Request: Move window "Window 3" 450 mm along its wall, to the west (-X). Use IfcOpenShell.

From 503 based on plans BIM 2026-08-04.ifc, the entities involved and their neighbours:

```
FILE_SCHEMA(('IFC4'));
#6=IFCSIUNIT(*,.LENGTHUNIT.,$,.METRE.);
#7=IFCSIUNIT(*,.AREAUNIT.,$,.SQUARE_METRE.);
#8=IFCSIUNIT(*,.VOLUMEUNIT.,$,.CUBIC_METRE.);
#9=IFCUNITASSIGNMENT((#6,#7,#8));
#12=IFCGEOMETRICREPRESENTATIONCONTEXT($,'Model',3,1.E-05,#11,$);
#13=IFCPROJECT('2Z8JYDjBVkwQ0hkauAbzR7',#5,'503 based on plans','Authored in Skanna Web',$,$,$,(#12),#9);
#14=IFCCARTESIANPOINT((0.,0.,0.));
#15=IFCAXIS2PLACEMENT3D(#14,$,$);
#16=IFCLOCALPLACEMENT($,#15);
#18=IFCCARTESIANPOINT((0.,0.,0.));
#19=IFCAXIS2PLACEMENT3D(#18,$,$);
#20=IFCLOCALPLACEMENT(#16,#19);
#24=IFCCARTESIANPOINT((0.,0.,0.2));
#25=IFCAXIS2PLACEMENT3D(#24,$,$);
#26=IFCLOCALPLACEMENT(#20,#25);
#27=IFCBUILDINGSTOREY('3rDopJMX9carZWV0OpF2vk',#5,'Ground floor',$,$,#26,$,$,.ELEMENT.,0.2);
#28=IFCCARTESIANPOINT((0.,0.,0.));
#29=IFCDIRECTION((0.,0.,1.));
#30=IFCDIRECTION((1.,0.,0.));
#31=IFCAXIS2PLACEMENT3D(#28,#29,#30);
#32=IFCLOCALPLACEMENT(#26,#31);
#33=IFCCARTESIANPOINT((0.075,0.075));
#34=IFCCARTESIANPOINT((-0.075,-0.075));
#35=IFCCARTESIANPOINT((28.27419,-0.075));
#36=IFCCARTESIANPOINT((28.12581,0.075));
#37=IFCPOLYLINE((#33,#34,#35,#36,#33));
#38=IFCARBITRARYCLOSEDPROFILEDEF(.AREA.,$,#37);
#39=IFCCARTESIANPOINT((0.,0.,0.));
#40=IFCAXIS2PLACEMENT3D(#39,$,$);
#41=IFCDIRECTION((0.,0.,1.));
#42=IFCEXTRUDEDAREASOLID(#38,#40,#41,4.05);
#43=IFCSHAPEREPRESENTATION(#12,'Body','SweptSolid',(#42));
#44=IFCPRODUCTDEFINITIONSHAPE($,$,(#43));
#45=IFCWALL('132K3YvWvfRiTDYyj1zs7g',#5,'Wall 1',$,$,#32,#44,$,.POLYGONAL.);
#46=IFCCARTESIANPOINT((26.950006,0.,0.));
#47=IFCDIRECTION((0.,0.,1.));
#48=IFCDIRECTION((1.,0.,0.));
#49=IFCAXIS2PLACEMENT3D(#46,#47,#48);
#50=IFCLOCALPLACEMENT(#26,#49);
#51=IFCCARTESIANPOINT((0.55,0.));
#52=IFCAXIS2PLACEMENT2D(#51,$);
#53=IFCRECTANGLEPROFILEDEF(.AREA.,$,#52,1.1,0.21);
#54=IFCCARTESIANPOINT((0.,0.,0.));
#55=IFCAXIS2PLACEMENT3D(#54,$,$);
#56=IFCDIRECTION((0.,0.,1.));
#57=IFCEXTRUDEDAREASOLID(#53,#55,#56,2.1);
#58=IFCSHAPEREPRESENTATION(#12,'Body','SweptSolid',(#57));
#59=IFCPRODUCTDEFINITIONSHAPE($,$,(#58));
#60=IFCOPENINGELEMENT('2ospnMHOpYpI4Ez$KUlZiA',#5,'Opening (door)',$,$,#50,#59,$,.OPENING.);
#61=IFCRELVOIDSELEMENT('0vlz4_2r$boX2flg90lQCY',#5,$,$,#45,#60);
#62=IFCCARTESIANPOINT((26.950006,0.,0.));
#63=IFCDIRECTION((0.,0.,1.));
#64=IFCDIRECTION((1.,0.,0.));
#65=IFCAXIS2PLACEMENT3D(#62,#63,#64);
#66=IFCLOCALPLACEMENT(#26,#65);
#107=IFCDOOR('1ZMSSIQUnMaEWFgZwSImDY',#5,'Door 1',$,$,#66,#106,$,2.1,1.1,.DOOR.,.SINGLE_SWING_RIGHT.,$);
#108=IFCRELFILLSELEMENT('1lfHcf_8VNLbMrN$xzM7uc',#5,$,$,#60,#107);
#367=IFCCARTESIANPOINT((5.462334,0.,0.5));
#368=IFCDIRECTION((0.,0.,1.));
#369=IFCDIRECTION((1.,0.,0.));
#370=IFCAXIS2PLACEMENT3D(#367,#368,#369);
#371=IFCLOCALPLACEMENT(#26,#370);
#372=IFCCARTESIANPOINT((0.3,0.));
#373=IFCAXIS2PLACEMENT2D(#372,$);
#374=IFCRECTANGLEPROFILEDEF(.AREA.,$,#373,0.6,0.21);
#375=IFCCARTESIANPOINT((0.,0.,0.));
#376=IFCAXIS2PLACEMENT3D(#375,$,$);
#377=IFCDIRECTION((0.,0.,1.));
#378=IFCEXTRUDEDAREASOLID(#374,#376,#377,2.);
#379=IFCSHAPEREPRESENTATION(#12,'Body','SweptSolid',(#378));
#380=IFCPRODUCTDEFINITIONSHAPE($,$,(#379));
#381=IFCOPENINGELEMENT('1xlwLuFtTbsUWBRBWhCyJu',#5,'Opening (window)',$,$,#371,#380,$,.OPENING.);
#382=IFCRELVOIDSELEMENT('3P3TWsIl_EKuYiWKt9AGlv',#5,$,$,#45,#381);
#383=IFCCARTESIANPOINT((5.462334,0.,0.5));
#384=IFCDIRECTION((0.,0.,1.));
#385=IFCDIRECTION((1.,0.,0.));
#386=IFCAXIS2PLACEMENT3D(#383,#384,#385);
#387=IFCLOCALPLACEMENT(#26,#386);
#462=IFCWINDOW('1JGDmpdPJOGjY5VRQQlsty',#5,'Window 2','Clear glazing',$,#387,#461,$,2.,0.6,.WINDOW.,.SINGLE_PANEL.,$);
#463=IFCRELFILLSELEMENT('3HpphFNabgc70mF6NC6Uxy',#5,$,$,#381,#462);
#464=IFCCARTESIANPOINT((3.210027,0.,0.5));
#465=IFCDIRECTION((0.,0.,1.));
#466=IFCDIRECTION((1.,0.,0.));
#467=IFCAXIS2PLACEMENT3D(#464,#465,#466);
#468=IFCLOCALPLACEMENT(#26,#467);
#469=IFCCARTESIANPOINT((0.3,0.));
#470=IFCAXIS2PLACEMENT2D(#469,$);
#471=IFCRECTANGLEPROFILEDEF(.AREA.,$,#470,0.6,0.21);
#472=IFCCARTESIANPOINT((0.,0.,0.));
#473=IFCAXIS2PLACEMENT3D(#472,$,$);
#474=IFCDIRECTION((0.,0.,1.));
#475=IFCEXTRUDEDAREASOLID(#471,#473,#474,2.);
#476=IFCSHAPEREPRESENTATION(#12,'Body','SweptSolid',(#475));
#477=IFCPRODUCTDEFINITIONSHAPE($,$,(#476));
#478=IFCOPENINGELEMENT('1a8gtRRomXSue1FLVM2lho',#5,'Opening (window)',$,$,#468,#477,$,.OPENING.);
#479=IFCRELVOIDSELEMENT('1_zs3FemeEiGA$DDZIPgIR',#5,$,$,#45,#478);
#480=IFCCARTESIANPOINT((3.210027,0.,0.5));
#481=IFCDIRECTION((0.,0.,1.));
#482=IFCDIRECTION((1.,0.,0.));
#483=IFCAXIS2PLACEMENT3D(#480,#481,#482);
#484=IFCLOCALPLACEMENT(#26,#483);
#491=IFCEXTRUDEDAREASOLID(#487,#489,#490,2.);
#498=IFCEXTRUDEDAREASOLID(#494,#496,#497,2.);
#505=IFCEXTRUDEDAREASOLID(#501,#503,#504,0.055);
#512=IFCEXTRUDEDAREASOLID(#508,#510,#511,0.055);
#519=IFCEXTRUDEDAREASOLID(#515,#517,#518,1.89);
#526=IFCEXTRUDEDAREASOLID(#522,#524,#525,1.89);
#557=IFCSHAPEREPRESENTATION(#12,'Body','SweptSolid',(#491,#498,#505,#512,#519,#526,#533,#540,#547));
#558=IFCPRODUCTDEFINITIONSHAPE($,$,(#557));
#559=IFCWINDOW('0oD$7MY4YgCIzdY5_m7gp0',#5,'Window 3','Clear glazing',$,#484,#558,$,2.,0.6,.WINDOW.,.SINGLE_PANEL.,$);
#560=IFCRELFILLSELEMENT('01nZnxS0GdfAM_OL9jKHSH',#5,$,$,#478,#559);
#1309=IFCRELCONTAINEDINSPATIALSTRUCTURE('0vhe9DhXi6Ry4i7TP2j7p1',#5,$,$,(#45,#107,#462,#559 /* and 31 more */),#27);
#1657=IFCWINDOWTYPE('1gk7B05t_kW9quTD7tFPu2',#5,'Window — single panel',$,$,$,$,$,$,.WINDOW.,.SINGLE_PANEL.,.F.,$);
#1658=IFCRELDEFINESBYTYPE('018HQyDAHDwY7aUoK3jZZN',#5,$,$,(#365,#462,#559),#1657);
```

```python
import ifcopenshell
import ifcopenshell.api.geometry
import ifcopenshell.util.placement
import ifcopenshell.util.unit

model = ifcopenshell.open("503 based on plans BIM 2026-08-04.ifc")
unit_scale = ifcopenshell.util.unit.calculate_unit_scale(model)

window = model.by_id(559)
opening = window.FillsVoids[0].RelatingOpeningElement
wall = opening.VoidsElements[0].RelatingBuildingElement

wall_matrix = ifcopenshell.util.placement.get_local_placement(wall.ObjectPlacement)
shift = wall_matrix[:3, 0] * -0.45 / unit_scale
before = ifcopenshell.util.placement.get_local_placement(window.ObjectPlacement)[:3, 3].copy()

# The window is not placed relative to its opening, so move both.
for product in (opening, window):
    matrix = ifcopenshell.util.placement.get_local_placement(product.ObjectPlacement)
    matrix[:3, 3] += shift
    ifcopenshell.api.geometry.edit_object_placement(model, product=product, matrix=matrix, is_si=False)

after = ifcopenshell.util.placement.get_local_placement(window.ObjectPlacement)[:3, 3]
print("window moved by", (after - before).round(3) + 0.0)

model.write("503 based on plans BIM 2026-08-04_updated.ifc")
```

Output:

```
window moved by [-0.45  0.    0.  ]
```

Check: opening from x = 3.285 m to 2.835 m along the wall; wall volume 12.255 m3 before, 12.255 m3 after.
